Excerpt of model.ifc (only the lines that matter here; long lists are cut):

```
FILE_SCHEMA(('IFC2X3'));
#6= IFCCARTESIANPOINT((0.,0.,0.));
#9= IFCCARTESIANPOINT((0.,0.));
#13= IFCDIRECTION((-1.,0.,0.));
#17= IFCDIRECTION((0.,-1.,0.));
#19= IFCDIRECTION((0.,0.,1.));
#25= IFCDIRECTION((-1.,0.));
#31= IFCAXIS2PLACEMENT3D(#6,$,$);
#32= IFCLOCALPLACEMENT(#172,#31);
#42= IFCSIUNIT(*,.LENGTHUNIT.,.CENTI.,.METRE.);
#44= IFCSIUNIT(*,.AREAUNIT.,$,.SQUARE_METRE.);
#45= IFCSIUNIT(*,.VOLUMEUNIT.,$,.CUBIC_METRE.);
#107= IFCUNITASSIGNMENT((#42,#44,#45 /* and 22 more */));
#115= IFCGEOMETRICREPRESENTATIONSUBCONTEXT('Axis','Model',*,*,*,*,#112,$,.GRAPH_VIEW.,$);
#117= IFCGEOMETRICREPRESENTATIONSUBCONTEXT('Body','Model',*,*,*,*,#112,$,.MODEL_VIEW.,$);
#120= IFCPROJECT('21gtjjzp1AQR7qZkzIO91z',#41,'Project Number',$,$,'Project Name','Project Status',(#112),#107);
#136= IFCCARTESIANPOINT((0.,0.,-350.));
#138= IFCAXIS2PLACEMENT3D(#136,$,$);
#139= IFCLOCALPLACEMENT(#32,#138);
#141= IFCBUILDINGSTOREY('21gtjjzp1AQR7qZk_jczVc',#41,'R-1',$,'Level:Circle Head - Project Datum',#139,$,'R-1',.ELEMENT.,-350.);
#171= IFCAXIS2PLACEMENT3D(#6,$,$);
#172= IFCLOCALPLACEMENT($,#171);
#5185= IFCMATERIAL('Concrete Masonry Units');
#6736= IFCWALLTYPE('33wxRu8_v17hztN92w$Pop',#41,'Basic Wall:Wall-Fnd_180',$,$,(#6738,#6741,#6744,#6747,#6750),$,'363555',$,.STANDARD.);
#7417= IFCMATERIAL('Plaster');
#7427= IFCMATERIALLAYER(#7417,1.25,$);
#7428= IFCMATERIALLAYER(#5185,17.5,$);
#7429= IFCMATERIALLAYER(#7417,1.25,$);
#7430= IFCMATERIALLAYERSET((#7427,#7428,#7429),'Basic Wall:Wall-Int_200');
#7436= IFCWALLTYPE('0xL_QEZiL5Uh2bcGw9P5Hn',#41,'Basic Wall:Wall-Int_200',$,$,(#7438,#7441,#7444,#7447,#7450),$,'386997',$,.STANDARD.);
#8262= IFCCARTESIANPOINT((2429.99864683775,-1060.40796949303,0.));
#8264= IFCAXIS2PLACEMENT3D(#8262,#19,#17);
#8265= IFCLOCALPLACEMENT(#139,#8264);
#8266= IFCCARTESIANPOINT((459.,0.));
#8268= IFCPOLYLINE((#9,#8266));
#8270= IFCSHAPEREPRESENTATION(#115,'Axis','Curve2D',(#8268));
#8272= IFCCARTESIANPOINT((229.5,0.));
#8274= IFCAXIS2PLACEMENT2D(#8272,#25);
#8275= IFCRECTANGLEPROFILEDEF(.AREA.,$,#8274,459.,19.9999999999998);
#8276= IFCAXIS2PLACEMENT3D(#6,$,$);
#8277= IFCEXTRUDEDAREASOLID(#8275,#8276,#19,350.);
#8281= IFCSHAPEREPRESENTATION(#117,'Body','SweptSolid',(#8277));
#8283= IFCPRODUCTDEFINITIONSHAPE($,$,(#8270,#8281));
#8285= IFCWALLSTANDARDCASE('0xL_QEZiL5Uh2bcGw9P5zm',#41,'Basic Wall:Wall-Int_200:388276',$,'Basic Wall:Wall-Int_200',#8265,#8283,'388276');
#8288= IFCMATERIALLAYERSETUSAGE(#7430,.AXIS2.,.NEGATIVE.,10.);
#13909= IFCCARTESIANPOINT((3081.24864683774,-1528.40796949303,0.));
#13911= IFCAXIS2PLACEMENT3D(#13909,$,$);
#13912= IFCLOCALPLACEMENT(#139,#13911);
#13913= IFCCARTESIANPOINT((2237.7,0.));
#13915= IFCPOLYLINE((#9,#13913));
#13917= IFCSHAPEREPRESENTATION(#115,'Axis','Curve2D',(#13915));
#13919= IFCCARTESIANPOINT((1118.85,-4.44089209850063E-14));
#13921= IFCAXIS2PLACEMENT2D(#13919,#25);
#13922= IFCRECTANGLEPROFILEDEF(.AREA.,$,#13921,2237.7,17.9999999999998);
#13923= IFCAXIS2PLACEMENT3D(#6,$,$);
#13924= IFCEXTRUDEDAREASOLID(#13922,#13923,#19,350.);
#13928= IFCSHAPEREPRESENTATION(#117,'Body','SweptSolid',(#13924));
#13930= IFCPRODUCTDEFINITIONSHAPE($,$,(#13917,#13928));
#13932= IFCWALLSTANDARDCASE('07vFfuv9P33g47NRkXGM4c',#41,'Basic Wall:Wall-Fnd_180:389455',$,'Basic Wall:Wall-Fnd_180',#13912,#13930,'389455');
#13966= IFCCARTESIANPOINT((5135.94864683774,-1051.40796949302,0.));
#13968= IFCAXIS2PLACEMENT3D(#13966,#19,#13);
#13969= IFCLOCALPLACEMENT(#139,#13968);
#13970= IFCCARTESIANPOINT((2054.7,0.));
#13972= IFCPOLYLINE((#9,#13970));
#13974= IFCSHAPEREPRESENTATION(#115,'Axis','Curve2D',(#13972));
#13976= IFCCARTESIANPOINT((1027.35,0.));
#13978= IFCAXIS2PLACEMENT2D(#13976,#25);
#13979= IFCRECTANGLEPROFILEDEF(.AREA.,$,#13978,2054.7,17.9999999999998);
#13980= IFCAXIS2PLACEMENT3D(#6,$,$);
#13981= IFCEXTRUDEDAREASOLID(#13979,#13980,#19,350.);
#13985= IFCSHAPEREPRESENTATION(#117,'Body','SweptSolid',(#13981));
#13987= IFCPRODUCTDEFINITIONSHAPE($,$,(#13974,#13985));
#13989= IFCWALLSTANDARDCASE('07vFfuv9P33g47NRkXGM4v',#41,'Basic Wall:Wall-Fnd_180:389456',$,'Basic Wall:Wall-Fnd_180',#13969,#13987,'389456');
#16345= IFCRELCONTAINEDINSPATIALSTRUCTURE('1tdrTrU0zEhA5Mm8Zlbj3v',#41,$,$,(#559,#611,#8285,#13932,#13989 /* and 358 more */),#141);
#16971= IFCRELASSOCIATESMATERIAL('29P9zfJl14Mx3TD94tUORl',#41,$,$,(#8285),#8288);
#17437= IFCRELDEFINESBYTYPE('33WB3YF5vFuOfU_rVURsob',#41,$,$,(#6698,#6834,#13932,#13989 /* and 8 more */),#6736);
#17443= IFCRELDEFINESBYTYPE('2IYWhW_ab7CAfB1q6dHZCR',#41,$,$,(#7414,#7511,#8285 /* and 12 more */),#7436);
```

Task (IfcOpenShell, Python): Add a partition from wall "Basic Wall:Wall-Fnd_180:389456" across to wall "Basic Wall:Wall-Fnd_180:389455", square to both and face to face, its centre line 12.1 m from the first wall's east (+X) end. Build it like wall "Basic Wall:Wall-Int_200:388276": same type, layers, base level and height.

```python
import numpy as np
import ifcopenshell
import ifcopenshell.api.geometry
import ifcopenshell.api.material
import ifcopenshell.api.pset
import ifcopenshell.api.root
import ifcopenshell.api.spatial
import ifcopenshell.api.type
import ifcopenshell.geom
import ifcopenshell.util.element
import ifcopenshell.util.placement
import ifcopenshell.util.representation
import ifcopenshell.util.shape
import ifcopenshell.util.unit

model = ifcopenshell.open("model.ifc")
unit_scale = ifcopenshell.util.unit.calculate_unit_scale(model)
settings = ifcopenshell.geom.settings()
settings.set("use-world-coords", True)

start_wall = model.by_guid("07vFfuv9P33g47NRkXGM4v")
end_wall = model.by_guid("07vFfuv9P33g47NRkXGM4c")
like = model.by_id(8285)
matrix = ifcopenshell.util.placement.get_local_placement(start_wall.ObjectPlacement)
matrix[:3, 3] *= unit_scale


def extent(element):
    """Bounding box in the first wall's axes, in metres."""
    shape = ifcopenshell.geom.create_shape(settings, element)
    points = (ifcopenshell.util.shape.get_vertices(shape.geometry) - matrix[:3, 3]) @ matrix[:3, :3]
    return points.min(axis=0), points.max(axis=0)


y_start = extent(start_wall)[1][1]
y_end = extent(end_wall)[0][1]
like_min, like_max = extent(like)
length, height = float(abs(y_end - y_start)), float(like_max[2] - like_min[2])
layer_set = ifcopenshell.util.element.get_material(like, should_skip_usage=True)
thickness = sum(layer.LayerThickness for layer in layer_set.MaterialLayers) * unit_scale

wall = ifcopenshell.api.root.create_entity(model, ifc_class="IfcWallStandardCase", name="New partition")
storey = ifcopenshell.util.element.get_container(like)
ifcopenshell.api.spatial.assign_container(model, products=[wall], relating_structure=storey)
ifcopenshell.api.type.assign_type(
    model, related_objects=[wall], relating_type=ifcopenshell.util.element.get_type(like), should_map_representations=False
)
rel = ifcopenshell.api.material.assign_material(
    model, products=[wall], type="IfcMaterialLayerSetUsage", material=layer_set
)
rel.RelatingMaterial.OffsetFromReferenceLine = -thickness / 2 / unit_scale
pset = ifcopenshell.api.pset.add_pset(model, product=wall, name="Pset_WallCommon")
ifcopenshell.api.pset.edit_pset(model, pset=pset, properties={"IsExternal": False, "LoadBearing": False})

# The axis runs down the middle of the wall.
axis = ifcopenshell.api.geometry.add_axis_representation(
    model, context=ifcopenshell.util.representation.get_context(model, "Model", "Axis"), axis=[(0.0, 0.0), (length, 0.0)]
)
body = ifcopenshell.api.geometry.add_wall_representation(
    model,
    context=ifcopenshell.util.representation.get_context(model, "Model", "Body", "MODEL_VIEW"),
    length=length,
    height=height,
    thickness=thickness,
    offset=-thickness / 2,
)
for representation in (axis, body):
    ifcopenshell.api.geometry.assign_representation(model, product=wall, representation=representation)

placement = matrix @ ifcopenshell.util.placement.rotation(90, "Z")
placement[:, 3] = matrix @ np.array([extent(start_wall)[0][0] + 12.1, y_start, like_min[2], 1.0])
ifcopenshell.api.geometry.edit_object_placement(model, product=wall, matrix=placement)

print(f"partition {length:.3f} m long, {height:.3f} m high, {thickness:.3f} m thick")

model.write("model_rev.ifc")
```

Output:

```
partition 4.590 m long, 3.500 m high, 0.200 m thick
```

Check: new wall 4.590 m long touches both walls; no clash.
